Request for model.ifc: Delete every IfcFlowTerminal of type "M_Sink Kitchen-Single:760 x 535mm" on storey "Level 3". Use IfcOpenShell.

First a look at what the model holds.

```python
import ifcopenshell
import ifcopenshell.util.element

model = ifcopenshell.open("model.ifc")
print(model.schema)
storey = next(s for s in model.by_type("IfcBuildingStorey") if s.Name == "Level 3")
terminals = [e for e in ifcopenshell.util.element.get_decomposition(storey) if e.is_a("IfcFlowTerminal")]
seen = {}
for e in terminals:
    element_type = ifcopenshell.util.element.get_type(e)
    name = element_type.Name if element_type not in (None, e) else None
    seen[name] = seen.get(name, 0) + 1
for name, count in sorted(seen.items(), key=str):
    print(count, "x", name)
```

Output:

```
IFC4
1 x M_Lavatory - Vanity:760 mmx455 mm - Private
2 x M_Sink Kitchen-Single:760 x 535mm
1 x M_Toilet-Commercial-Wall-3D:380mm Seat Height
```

```python
import ifcopenshell
import ifcopenshell.api.root
import ifcopenshell.util.element

model = ifcopenshell.open("model.ifc")

storey = next(s for s in model.by_type("IfcBuildingStorey") if s.Name == "Level 3")
terminals = [e for e in ifcopenshell.util.element.get_decomposition(storey) if e.is_a("IfcFlowTerminal")]
targets = [e for e in terminals if (t := ifcopenshell.util.element.get_type(e)) not in (None, e) and t.Name == "M_Sink Kitchen-Single:760 x 535mm"]

for e in targets:
    ifcopenshell.api.root.remove_product(model, product=e)
print(len(targets), "removed")

model.write("model_rev.ifc")
```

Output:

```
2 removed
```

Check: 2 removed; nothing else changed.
